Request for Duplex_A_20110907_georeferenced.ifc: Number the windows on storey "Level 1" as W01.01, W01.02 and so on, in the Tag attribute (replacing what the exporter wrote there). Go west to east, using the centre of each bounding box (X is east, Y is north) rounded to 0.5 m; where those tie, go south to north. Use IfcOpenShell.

First a look at what the model holds.

```python
import ifcopenshell
import ifcopenshell.util.element
import ifcopenshell.util.placement

model = ifcopenshell.open("Duplex_A_20110907_georeferenced.ifc")
print(model.schema)
storey = next(s for s in model.by_type("IfcBuildingStorey") if s.Name == "Level 1")
windows = [e for e in ifcopenshell.util.element.get_decomposition(storey) if e.is_a("IfcWindow")]
for e in sorted(windows, key=lambda e: e.id()):
    origin = ifcopenshell.util.placement.get_local_placement(e.ObjectPlacement)[:3, 3]
    print(e.id(), e.Tag, e.Name, origin.round(2) + 0.0, sep=" | ")
```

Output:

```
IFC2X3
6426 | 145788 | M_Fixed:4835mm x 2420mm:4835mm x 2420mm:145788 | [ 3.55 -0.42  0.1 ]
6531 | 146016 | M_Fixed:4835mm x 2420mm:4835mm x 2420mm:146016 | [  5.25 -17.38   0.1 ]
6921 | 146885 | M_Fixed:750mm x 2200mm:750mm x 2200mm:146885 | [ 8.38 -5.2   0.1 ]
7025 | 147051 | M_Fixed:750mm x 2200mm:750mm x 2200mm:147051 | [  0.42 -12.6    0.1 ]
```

```python
import ifcopenshell
import ifcopenshell.geom
import ifcopenshell.util.element
import ifcopenshell.util.shape

model = ifcopenshell.open("Duplex_A_20110907_georeferenced.ifc")
settings = ifcopenshell.geom.settings()
settings.set("use-world-coords", True)


def centre(element):
    shape = ifcopenshell.geom.create_shape(settings, element)
    return ifcopenshell.util.shape.get_bbox_centroid(shape.geometry)


storey = next(s for s in model.by_type("IfcBuildingStorey") if s.Name == "Level 1")
windows = [e for e in ifcopenshell.util.element.get_decomposition(storey) if e.is_a("IfcWindow")]

# Insertion points can sit at a corner or the storey origin, so sort by the geometry (in metres).
centres = {e: centre(e) for e in windows}
windows.sort(key=lambda e: (round(centres[e][0] / 0.5), centres[e][1]))

for i, e in enumerate(windows, start=1):
    number = f"W01.{i:02d}"
    e.Tag = number
    print(e.id(), number)

model.write("Duplex_A_20110907_georeferenced_rev.ifc")
```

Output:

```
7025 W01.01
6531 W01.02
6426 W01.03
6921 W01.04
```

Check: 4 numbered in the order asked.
